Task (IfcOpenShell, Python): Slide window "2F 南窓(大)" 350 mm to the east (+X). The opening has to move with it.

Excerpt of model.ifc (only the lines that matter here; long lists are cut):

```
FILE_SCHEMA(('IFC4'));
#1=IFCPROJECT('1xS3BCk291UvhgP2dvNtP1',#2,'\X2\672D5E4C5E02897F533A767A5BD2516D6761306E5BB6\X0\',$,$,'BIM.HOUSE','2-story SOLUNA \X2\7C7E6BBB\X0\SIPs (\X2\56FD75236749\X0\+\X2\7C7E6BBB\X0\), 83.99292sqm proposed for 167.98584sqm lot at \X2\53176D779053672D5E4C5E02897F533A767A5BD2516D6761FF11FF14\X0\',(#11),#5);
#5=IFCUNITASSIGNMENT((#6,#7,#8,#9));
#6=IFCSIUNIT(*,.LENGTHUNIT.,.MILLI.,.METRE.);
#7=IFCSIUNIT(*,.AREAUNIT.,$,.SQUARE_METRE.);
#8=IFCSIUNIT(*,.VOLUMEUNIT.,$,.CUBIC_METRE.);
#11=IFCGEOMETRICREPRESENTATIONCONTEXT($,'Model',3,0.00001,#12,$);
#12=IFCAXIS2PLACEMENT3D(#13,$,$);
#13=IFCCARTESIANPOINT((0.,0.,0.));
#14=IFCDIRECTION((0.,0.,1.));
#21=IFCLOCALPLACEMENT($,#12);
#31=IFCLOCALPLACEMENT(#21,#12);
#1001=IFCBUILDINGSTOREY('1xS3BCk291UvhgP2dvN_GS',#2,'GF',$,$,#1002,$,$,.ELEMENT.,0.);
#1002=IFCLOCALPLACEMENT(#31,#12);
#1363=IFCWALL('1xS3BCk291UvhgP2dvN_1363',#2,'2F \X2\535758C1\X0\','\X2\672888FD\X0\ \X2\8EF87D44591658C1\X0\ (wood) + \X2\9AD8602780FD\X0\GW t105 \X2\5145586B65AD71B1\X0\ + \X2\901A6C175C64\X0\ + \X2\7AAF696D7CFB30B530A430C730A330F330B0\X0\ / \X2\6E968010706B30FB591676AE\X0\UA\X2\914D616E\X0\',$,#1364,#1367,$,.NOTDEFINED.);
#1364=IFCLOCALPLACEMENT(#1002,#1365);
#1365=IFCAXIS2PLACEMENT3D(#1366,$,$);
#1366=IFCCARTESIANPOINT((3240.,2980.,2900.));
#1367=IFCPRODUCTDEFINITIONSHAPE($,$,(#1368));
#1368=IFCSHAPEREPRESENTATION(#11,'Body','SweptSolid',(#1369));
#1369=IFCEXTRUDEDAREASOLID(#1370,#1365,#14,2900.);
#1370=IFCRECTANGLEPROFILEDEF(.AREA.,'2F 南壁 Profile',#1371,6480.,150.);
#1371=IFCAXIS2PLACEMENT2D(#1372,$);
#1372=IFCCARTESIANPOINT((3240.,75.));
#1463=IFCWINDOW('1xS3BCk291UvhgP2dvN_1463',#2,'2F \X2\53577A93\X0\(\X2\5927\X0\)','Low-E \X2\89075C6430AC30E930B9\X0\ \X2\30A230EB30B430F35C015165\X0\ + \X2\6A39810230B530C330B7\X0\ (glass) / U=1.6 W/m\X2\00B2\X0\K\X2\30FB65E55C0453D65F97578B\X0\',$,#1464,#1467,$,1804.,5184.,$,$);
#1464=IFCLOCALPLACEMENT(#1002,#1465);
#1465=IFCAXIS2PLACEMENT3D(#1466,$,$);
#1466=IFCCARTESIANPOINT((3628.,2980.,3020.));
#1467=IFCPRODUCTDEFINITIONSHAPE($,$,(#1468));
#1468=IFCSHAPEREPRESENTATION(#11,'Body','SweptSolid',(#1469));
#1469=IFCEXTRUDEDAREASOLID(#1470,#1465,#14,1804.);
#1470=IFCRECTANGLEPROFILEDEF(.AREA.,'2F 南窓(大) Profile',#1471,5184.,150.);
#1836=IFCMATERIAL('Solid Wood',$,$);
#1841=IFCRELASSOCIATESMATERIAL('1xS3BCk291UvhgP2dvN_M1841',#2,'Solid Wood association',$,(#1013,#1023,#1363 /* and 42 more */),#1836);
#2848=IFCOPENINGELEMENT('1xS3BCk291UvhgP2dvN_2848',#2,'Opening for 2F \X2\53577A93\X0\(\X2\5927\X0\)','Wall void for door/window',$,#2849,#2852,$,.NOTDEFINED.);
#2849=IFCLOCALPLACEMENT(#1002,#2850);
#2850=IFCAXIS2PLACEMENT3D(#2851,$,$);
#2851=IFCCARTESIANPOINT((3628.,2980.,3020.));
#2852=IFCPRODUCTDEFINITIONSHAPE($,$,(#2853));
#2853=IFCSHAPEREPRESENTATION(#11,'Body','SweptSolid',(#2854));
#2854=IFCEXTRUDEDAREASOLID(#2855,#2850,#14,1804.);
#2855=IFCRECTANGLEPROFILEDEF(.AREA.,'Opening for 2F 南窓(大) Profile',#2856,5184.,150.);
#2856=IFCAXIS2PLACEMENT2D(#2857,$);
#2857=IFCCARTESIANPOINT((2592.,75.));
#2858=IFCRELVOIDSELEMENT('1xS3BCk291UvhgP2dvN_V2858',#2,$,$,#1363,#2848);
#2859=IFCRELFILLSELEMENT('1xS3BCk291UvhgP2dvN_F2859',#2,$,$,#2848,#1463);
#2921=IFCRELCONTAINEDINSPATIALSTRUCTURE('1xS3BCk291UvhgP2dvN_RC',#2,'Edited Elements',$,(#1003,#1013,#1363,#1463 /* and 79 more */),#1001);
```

```python
import ifcopenshell
import ifcopenshell.api.geometry
import ifcopenshell.util.placement

model = ifcopenshell.open("model.ifc")

window = model.by_guid("1xS3BCk291UvhgP2dvN_1463")
opening = window.FillsVoids[0].RelatingOpeningElement
wall = opening.VoidsElements[0].RelatingBuildingElement

wall_matrix = ifcopenshell.util.placement.get_local_placement(wall.ObjectPlacement)
shift = wall_matrix[:3, 0] * 350.0
before = ifcopenshell.util.placement.get_local_placement(window.ObjectPlacement)[:3, 3].copy()

# The window is not placed relative to its opening, so move both.
for product in (opening, window):
    matrix = ifcopenshell.util.placement.get_local_placement(product.ObjectPlacement)
    matrix[:3, 3] += shift
    ifcopenshell.api.geometry.edit_object_placement(model, product=product, matrix=matrix, is_si=False)

after = ifcopenshell.util.placement.get_local_placement(window.ObjectPlacement)[:3, 3]
print("window moved by", (after - before).round(3) + 0.0)

model.write("model_updated.ifc")
```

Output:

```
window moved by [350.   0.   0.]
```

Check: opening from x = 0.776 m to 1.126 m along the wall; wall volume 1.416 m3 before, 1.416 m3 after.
